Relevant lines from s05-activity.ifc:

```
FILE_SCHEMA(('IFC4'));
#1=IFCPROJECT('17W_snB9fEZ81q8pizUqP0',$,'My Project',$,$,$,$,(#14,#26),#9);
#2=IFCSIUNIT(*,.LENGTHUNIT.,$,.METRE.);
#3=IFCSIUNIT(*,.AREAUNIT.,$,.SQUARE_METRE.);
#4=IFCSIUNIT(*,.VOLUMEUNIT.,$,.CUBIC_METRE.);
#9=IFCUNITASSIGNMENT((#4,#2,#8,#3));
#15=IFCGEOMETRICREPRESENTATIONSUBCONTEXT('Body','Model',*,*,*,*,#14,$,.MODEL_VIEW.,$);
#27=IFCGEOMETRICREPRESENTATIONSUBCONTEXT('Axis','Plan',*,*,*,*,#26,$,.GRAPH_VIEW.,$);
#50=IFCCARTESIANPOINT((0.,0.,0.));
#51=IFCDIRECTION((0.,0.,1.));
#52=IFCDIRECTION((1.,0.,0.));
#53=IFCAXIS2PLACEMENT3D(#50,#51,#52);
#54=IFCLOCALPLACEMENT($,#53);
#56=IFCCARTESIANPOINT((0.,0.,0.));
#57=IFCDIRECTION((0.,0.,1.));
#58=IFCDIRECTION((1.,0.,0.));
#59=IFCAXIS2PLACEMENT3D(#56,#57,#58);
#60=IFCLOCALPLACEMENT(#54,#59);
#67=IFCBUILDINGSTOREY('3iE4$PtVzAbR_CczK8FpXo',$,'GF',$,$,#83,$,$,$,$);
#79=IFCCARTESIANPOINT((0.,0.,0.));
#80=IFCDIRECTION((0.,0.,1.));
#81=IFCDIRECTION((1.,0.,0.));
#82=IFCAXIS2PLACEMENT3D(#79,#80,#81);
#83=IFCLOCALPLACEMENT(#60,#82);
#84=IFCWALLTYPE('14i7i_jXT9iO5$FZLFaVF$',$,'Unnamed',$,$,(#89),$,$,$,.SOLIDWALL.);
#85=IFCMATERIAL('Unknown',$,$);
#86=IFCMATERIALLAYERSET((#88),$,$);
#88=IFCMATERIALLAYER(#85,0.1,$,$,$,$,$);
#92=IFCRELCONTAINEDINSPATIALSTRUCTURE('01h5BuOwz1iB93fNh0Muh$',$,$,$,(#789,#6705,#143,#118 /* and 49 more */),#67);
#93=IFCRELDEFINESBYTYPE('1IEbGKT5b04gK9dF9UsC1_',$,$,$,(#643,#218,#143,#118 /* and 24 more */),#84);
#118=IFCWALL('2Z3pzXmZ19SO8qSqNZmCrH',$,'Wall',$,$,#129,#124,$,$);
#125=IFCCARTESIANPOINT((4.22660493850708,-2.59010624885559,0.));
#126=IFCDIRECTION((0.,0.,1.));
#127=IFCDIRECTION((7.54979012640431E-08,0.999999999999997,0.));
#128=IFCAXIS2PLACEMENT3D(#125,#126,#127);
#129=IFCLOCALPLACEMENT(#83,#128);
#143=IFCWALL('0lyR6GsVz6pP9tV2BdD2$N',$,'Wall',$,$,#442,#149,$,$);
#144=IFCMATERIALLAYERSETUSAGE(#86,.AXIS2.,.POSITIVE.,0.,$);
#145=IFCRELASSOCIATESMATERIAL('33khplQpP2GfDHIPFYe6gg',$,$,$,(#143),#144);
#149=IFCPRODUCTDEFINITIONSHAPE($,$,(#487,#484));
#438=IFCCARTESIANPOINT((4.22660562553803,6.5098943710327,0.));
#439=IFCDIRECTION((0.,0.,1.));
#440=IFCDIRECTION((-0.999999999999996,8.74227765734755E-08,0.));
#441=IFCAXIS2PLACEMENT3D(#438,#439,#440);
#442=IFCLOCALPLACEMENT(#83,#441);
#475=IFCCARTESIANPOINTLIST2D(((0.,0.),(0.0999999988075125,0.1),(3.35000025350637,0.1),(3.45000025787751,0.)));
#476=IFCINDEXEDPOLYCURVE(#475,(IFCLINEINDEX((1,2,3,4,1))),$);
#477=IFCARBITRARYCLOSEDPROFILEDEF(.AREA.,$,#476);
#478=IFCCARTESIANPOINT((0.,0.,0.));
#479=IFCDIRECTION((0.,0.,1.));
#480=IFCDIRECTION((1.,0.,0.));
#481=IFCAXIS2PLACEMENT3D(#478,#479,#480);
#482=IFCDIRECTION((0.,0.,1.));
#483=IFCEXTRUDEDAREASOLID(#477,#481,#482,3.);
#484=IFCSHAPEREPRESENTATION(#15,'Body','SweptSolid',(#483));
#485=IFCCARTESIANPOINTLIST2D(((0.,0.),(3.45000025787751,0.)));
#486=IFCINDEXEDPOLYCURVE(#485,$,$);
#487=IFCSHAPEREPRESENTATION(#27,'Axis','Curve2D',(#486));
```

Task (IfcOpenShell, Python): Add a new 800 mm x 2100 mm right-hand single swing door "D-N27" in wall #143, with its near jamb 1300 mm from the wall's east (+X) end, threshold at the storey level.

```python
import numpy as np
import ifcopenshell
import ifcopenshell.api.feature
import ifcopenshell.api.geometry
import ifcopenshell.api.root
import ifcopenshell.api.spatial
import ifcopenshell.geom
import ifcopenshell.util.element
import ifcopenshell.util.placement
import ifcopenshell.util.representation
import ifcopenshell.util.shape
import ifcopenshell.util.unit

model = ifcopenshell.open("s05-activity.ifc")
unit_scale = ifcopenshell.util.unit.calculate_unit_scale(model)
settings = ifcopenshell.geom.settings()


def volume(element):
    """Net volume in cubic metres, openings subtracted."""
    shape = ifcopenshell.geom.create_shape(settings, element)
    return ifcopenshell.util.shape.get_volume(shape.geometry)


wall = model.by_guid("0lyR6GsVz6pP9tV2BdD2$N")
storey = ifcopenshell.util.element.get_container(wall, ifc_class="IfcBuildingStorey")
context = ifcopenshell.util.representation.get_context(model, "Model", "Body", "MODEL_VIEW")
before = volume(wall)

width, height, from_end, sill = 0.8, 2.1, 1.3, 0.0  # metres

# The wall runs along its own X axis, and the end named is its -X end.
wall_shape = ifcopenshell.geom.create_shape(settings, wall)
x, y, z = ifcopenshell.util.shape.get_vertices(wall_shape.geometry).T
start = x.min() + from_end
face, thickness = float(y.min()), float(y.max() - y.min())
wall_matrix = ifcopenshell.util.placement.get_local_placement(wall.ObjectPlacement)
level = ifcopenshell.util.placement.get_local_placement(storey.ObjectPlacement)[2, 3]


def in_wall(x, y):
    """Placement at x, y metres in the wall's axes, at sill height."""
    matrix = wall_matrix.copy()
    matrix[:, 3] = wall_matrix @ np.array([x / unit_scale, y / unit_scale, 0.0, 1.0])
    matrix[2, 3] = level + sill / unit_scale
    return matrix


# Opening: a box that overshoots both wall faces by 50 mm.
opening = ifcopenshell.api.root.create_entity(model, ifc_class="IfcOpeningElement", predefined_type="OPENING")
box = ifcopenshell.api.geometry.add_wall_representation(
    model, context=context, length=width, height=height, thickness=thickness + 0.1
)
ifcopenshell.api.geometry.assign_representation(model, product=opening, representation=box)
ifcopenshell.api.geometry.edit_object_placement(model, product=opening, matrix=in_wall(start, face - 0.05), is_si=False)
ifcopenshell.api.feature.add_feature(model, feature=opening, element=wall)

door = ifcopenshell.api.root.create_entity(model, ifc_class="IfcDoor", name="D-N27", predefined_type="DOOR")
door.OverallWidth, door.OverallHeight = width / unit_scale, height / unit_scale
door.OperationType = "SINGLE_SWING_RIGHT"
body = ifcopenshell.api.geometry.add_door_representation(
    model,
    context=context,
    overall_width=door.OverallWidth,
    overall_height=door.OverallHeight,
    operation_type="SINGLE_SWING_RIGHT",
    lining_properties={"LiningDepth": thickness / unit_scale, "ThresholdDepth": thickness / unit_scale},
)
ifcopenshell.api.geometry.assign_representation(model, product=door, representation=body)
ifcopenshell.api.spatial.assign_container(model, products=[door], relating_structure=storey)
ifcopenshell.api.feature.add_filling(model, opening=opening, element=door)

# The lining spans the wall, so the door starts at the wall face.
ifcopenshell.api.geometry.edit_object_placement(model, product=door, matrix=in_wall(start, face), is_si=False)

after = volume(wall)

print(f"wall volume {before:.3f} -> {after:.3f} m3")

model.write("s05-activity_v2.ifc")
```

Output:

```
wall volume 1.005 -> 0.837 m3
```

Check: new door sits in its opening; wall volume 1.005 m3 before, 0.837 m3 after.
